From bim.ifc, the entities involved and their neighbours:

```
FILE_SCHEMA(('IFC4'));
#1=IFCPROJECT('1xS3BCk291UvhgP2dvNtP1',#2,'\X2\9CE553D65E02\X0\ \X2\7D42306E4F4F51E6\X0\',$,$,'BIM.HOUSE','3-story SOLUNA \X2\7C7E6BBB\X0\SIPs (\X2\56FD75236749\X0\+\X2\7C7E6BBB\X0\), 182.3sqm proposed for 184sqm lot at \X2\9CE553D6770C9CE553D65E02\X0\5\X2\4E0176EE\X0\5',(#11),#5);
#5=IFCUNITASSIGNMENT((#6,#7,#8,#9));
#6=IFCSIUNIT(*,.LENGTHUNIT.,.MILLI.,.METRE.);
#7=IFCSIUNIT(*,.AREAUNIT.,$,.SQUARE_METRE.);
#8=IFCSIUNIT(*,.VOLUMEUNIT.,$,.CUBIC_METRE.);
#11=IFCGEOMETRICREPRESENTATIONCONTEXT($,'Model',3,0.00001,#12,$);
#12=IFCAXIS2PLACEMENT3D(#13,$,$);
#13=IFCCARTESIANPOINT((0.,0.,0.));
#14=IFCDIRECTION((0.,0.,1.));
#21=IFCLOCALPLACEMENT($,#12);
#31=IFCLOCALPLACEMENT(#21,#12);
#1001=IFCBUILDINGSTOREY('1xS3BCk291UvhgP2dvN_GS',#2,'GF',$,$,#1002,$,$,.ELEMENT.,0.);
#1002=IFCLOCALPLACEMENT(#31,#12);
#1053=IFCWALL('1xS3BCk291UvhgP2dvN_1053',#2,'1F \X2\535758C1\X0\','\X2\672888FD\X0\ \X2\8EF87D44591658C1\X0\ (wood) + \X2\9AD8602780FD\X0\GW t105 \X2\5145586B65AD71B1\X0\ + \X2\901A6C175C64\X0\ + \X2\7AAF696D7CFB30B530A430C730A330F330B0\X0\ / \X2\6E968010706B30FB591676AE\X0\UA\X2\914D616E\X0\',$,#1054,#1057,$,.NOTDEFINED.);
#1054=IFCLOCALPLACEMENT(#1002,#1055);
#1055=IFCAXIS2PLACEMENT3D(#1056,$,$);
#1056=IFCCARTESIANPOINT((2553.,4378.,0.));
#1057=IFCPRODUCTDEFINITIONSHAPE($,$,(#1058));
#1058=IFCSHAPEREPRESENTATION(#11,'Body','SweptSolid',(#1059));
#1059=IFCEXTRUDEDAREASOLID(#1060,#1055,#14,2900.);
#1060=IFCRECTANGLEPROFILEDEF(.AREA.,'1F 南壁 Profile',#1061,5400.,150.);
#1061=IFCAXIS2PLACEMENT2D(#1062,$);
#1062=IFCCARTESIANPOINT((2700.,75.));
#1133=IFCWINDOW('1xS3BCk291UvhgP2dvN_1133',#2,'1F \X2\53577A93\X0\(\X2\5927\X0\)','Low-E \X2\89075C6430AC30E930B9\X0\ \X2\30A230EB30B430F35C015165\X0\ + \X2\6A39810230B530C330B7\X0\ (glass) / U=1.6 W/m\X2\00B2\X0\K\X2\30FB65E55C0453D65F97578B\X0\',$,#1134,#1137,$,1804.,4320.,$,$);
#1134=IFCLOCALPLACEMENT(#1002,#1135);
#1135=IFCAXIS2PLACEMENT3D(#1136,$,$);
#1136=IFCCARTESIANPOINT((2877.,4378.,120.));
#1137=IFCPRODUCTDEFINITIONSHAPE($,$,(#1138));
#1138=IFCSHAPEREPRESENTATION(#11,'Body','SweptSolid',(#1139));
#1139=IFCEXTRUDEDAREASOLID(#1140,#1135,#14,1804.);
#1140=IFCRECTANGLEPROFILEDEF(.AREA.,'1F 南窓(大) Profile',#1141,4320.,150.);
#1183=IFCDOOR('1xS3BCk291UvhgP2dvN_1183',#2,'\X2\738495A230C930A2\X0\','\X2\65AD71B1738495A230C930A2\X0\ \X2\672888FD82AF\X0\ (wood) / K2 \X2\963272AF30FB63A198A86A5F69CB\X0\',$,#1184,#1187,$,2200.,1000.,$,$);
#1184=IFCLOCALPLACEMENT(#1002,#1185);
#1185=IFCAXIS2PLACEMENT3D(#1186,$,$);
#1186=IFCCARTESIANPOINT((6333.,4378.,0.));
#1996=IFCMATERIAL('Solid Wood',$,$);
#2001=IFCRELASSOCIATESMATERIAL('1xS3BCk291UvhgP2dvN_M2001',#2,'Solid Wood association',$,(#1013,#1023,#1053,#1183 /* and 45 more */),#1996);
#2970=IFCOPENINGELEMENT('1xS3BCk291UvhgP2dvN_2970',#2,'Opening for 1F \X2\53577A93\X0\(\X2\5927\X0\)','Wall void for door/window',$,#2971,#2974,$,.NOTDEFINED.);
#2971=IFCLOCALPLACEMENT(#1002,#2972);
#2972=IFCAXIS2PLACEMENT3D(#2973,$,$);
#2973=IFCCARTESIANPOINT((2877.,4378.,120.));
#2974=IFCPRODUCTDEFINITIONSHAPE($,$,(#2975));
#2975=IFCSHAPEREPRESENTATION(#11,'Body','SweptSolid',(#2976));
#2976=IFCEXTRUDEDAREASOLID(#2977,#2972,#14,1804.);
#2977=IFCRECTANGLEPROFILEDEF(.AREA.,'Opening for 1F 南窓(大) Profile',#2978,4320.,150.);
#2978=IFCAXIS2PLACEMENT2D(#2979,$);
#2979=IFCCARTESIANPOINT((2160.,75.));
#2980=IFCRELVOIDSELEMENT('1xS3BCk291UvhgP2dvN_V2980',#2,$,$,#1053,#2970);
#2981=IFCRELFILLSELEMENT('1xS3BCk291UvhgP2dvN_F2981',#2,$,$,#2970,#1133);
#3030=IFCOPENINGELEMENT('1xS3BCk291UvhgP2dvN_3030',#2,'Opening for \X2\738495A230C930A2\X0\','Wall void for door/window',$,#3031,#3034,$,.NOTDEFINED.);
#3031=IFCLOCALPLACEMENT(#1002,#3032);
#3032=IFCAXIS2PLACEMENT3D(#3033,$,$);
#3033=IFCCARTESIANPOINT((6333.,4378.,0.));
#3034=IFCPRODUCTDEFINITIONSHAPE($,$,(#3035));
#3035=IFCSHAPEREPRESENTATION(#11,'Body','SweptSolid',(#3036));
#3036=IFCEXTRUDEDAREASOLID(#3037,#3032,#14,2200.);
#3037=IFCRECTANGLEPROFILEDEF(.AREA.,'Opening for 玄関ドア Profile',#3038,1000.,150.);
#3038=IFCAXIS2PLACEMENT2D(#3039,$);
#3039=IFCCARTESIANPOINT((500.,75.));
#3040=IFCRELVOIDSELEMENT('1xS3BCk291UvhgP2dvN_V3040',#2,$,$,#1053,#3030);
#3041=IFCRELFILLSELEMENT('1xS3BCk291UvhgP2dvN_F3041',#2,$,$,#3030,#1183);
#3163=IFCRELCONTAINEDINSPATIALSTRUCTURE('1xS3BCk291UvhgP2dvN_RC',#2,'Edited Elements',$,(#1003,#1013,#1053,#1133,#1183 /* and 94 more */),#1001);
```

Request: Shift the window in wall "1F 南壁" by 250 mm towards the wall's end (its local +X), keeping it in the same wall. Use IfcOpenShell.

```python
import ifcopenshell
import ifcopenshell.api.geometry
import ifcopenshell.util.placement
import ifcopenshell.util.unit

model = ifcopenshell.open("bim.ifc")
unit_scale = ifcopenshell.util.unit.calculate_unit_scale(model)

window = model.by_guid("1xS3BCk291UvhgP2dvN_1133")
opening = window.FillsVoids[0].RelatingOpeningElement
wall = opening.VoidsElements[0].RelatingBuildingElement

wall_matrix = ifcopenshell.util.placement.get_local_placement(wall.ObjectPlacement)
shift = wall_matrix[:3, 0] * 0.25 / unit_scale
before = ifcopenshell.util.placement.get_local_placement(window.ObjectPlacement)[:3, 3].copy()

# The window is not placed relative to its opening, so move both.
for product in (opening, window):
    matrix = ifcopenshell.util.placement.get_local_placement(product.ObjectPlacement)
    matrix[:3, 3] += shift
    ifcopenshell.api.geometry.edit_object_placement(model, product=product, matrix=matrix, is_si=False)

after = ifcopenshell.util.placement.get_local_placement(window.ObjectPlacement)[:3, 3]
print("window moved by", (after - before).round(3) + 0.0)

model.write("bim_rev.ifc")
```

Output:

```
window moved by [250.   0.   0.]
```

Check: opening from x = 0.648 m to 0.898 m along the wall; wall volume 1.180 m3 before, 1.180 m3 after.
